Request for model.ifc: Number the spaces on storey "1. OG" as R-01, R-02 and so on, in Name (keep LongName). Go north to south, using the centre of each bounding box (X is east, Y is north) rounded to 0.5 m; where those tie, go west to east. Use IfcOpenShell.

First a look at what the model holds.

```python
import ifcopenshell
import ifcopenshell.util.element
import ifcopenshell.util.placement

model = ifcopenshell.open("model.ifc")
print(model.schema)
storey = next(s for s in model.by_type("IfcBuildingStorey") if s.Name == "1. OG")
spaces = [e for e in ifcopenshell.util.element.get_decomposition(storey) if e.is_a("IfcSpace")]
for e in sorted(spaces, key=lambda e: e.id()):
    origin = ifcopenshell.util.placement.get_local_placement(e.ObjectPlacement)[:3, 3]
    print(e.id(), e.Name, e.LongName, origin.round(2) + 0.0, sep=" | ")
```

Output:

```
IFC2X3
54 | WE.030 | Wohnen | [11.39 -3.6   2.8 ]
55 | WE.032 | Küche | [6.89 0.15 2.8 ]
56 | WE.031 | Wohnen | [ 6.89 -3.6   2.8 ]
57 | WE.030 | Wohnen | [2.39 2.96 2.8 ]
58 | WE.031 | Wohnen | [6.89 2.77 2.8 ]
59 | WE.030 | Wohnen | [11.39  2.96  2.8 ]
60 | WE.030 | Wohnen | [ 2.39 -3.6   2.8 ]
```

```python
import ifcopenshell
import ifcopenshell.geom
import ifcopenshell.util.element
import ifcopenshell.util.shape

model = ifcopenshell.open("model.ifc")
settings = ifcopenshell.geom.settings()
settings.set("use-world-coords", True)


def centre(element):
    shape = ifcopenshell.geom.create_shape(settings, element)
    return ifcopenshell.util.shape.get_bbox_centroid(shape.geometry)


storey = next(s for s in model.by_type("IfcBuildingStorey") if s.Name == "1. OG")
spaces = [e for e in ifcopenshell.util.element.get_decomposition(storey) if e.is_a("IfcSpace")]

# Insertion points can sit at a corner or the storey origin, so sort by the geometry (in metres).
centres = {e: centre(e) for e in spaces}
spaces.sort(key=lambda e: (-round(centres[e][1] / 0.5), centres[e][0]))

for i, e in enumerate(spaces, start=1):
    number = f"R-{i:02d}"
    e.Name = number
    print(e.id(), number)

model.write("model_updated.ifc")
```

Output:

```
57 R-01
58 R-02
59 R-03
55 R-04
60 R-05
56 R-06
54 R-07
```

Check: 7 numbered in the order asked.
